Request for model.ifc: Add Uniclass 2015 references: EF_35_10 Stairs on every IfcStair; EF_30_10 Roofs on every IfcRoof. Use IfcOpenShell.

First a look at what the model holds.

```python
import ifcopenshell

model = ifcopenshell.open("model.ifc")
print(model.schema)
print("classifications:", [c.Name for c in model.by_type("IfcClassification")])
for ifc_class in ("IfcDoor", "IfcRoof", "IfcStair", "IfcWall", "IfcWindow"):
    print(ifc_class, len(model.by_type(ifc_class)))
```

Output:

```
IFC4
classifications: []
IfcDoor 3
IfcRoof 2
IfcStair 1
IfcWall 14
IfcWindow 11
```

```python
import ifcopenshell
import ifcopenshell.api.classification

model = ifcopenshell.open("model.ifc")

system = ifcopenshell.api.classification.add_classification(model, classification="Uniclass 2015")

codes = {
    "IfcStair": ("EF_35_10", "Stairs"),
    "IfcRoof": ("EF_30_10", "Roofs"),
}
for ifc_class, (code, name) in codes.items():
    products = model.by_type(ifc_class)
    ifcopenshell.api.classification.add_reference(
        model, products=products, classification=system, identification=code, name=name
    )
    print(code, len(products))

model.write("model_rev.ifc")
```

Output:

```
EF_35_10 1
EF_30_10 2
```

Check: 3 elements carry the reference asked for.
